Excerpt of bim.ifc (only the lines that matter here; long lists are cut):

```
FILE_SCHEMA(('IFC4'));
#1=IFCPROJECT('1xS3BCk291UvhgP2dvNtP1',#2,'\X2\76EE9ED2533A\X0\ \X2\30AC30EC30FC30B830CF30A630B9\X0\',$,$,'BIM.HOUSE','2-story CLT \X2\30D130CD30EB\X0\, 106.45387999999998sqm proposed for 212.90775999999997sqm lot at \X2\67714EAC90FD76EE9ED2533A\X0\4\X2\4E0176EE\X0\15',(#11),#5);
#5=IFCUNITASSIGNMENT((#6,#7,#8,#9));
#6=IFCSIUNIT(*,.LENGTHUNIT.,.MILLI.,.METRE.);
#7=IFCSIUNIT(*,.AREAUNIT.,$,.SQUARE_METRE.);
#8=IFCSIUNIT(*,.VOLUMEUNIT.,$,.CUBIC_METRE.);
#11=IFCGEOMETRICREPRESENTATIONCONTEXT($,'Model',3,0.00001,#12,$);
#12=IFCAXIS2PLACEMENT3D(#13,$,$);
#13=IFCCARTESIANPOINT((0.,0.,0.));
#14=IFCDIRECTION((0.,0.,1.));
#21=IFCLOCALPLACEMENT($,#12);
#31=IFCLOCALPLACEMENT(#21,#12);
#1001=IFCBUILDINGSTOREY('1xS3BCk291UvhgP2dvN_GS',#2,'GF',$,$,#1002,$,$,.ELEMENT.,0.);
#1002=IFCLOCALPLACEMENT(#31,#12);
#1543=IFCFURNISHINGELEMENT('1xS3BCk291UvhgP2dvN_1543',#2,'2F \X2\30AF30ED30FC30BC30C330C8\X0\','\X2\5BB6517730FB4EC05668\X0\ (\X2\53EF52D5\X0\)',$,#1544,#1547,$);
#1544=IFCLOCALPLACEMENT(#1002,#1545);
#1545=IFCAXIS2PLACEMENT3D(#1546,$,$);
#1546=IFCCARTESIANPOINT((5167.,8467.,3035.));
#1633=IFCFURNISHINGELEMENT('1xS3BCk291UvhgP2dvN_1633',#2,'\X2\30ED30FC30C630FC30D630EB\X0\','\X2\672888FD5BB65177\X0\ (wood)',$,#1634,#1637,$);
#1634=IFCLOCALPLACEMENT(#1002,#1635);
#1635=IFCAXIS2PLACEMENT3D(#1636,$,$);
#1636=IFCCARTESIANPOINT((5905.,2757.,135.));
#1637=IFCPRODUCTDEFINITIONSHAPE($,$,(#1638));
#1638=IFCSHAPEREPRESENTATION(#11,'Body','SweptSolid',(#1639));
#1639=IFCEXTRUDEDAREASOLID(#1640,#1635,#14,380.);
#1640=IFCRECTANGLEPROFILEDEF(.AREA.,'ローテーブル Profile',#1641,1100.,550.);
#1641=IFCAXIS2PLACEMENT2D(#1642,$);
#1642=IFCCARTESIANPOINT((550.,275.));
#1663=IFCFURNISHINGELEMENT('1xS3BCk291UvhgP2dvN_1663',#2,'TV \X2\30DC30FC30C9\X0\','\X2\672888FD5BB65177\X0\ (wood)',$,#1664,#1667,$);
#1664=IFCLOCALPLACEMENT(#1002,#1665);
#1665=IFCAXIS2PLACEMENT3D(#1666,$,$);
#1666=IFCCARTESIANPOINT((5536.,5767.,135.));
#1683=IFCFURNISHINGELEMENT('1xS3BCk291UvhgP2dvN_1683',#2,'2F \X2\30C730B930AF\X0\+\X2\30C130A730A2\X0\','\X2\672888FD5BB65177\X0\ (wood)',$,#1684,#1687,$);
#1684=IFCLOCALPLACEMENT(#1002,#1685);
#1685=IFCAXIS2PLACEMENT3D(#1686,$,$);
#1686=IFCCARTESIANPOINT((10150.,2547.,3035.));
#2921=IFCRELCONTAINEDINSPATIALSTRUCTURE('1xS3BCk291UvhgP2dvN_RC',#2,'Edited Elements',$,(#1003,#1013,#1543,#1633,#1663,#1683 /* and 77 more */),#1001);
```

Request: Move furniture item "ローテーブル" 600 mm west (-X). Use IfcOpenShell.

```python
import ifcopenshell
import ifcopenshell.api.geometry
import ifcopenshell.util.placement
import ifcopenshell.util.unit

model = ifcopenshell.open("bim.ifc")
unit_scale = ifcopenshell.util.unit.calculate_unit_scale(model)

item = model.by_id(1633)
matrix = ifcopenshell.util.placement.get_local_placement(item.ObjectPlacement)
matrix[0, 3] -= 0.6 / unit_scale
ifcopenshell.api.geometry.edit_object_placement(model, product=item, matrix=matrix, is_si=False)

print(ifcopenshell.util.placement.get_local_placement(item.ObjectPlacement).round(3) + 0.0)

model.write("bim-out.ifc")
```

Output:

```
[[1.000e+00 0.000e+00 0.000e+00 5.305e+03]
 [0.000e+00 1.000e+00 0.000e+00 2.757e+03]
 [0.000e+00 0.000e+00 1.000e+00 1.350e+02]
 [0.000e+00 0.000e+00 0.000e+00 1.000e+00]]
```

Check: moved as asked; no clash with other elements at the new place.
